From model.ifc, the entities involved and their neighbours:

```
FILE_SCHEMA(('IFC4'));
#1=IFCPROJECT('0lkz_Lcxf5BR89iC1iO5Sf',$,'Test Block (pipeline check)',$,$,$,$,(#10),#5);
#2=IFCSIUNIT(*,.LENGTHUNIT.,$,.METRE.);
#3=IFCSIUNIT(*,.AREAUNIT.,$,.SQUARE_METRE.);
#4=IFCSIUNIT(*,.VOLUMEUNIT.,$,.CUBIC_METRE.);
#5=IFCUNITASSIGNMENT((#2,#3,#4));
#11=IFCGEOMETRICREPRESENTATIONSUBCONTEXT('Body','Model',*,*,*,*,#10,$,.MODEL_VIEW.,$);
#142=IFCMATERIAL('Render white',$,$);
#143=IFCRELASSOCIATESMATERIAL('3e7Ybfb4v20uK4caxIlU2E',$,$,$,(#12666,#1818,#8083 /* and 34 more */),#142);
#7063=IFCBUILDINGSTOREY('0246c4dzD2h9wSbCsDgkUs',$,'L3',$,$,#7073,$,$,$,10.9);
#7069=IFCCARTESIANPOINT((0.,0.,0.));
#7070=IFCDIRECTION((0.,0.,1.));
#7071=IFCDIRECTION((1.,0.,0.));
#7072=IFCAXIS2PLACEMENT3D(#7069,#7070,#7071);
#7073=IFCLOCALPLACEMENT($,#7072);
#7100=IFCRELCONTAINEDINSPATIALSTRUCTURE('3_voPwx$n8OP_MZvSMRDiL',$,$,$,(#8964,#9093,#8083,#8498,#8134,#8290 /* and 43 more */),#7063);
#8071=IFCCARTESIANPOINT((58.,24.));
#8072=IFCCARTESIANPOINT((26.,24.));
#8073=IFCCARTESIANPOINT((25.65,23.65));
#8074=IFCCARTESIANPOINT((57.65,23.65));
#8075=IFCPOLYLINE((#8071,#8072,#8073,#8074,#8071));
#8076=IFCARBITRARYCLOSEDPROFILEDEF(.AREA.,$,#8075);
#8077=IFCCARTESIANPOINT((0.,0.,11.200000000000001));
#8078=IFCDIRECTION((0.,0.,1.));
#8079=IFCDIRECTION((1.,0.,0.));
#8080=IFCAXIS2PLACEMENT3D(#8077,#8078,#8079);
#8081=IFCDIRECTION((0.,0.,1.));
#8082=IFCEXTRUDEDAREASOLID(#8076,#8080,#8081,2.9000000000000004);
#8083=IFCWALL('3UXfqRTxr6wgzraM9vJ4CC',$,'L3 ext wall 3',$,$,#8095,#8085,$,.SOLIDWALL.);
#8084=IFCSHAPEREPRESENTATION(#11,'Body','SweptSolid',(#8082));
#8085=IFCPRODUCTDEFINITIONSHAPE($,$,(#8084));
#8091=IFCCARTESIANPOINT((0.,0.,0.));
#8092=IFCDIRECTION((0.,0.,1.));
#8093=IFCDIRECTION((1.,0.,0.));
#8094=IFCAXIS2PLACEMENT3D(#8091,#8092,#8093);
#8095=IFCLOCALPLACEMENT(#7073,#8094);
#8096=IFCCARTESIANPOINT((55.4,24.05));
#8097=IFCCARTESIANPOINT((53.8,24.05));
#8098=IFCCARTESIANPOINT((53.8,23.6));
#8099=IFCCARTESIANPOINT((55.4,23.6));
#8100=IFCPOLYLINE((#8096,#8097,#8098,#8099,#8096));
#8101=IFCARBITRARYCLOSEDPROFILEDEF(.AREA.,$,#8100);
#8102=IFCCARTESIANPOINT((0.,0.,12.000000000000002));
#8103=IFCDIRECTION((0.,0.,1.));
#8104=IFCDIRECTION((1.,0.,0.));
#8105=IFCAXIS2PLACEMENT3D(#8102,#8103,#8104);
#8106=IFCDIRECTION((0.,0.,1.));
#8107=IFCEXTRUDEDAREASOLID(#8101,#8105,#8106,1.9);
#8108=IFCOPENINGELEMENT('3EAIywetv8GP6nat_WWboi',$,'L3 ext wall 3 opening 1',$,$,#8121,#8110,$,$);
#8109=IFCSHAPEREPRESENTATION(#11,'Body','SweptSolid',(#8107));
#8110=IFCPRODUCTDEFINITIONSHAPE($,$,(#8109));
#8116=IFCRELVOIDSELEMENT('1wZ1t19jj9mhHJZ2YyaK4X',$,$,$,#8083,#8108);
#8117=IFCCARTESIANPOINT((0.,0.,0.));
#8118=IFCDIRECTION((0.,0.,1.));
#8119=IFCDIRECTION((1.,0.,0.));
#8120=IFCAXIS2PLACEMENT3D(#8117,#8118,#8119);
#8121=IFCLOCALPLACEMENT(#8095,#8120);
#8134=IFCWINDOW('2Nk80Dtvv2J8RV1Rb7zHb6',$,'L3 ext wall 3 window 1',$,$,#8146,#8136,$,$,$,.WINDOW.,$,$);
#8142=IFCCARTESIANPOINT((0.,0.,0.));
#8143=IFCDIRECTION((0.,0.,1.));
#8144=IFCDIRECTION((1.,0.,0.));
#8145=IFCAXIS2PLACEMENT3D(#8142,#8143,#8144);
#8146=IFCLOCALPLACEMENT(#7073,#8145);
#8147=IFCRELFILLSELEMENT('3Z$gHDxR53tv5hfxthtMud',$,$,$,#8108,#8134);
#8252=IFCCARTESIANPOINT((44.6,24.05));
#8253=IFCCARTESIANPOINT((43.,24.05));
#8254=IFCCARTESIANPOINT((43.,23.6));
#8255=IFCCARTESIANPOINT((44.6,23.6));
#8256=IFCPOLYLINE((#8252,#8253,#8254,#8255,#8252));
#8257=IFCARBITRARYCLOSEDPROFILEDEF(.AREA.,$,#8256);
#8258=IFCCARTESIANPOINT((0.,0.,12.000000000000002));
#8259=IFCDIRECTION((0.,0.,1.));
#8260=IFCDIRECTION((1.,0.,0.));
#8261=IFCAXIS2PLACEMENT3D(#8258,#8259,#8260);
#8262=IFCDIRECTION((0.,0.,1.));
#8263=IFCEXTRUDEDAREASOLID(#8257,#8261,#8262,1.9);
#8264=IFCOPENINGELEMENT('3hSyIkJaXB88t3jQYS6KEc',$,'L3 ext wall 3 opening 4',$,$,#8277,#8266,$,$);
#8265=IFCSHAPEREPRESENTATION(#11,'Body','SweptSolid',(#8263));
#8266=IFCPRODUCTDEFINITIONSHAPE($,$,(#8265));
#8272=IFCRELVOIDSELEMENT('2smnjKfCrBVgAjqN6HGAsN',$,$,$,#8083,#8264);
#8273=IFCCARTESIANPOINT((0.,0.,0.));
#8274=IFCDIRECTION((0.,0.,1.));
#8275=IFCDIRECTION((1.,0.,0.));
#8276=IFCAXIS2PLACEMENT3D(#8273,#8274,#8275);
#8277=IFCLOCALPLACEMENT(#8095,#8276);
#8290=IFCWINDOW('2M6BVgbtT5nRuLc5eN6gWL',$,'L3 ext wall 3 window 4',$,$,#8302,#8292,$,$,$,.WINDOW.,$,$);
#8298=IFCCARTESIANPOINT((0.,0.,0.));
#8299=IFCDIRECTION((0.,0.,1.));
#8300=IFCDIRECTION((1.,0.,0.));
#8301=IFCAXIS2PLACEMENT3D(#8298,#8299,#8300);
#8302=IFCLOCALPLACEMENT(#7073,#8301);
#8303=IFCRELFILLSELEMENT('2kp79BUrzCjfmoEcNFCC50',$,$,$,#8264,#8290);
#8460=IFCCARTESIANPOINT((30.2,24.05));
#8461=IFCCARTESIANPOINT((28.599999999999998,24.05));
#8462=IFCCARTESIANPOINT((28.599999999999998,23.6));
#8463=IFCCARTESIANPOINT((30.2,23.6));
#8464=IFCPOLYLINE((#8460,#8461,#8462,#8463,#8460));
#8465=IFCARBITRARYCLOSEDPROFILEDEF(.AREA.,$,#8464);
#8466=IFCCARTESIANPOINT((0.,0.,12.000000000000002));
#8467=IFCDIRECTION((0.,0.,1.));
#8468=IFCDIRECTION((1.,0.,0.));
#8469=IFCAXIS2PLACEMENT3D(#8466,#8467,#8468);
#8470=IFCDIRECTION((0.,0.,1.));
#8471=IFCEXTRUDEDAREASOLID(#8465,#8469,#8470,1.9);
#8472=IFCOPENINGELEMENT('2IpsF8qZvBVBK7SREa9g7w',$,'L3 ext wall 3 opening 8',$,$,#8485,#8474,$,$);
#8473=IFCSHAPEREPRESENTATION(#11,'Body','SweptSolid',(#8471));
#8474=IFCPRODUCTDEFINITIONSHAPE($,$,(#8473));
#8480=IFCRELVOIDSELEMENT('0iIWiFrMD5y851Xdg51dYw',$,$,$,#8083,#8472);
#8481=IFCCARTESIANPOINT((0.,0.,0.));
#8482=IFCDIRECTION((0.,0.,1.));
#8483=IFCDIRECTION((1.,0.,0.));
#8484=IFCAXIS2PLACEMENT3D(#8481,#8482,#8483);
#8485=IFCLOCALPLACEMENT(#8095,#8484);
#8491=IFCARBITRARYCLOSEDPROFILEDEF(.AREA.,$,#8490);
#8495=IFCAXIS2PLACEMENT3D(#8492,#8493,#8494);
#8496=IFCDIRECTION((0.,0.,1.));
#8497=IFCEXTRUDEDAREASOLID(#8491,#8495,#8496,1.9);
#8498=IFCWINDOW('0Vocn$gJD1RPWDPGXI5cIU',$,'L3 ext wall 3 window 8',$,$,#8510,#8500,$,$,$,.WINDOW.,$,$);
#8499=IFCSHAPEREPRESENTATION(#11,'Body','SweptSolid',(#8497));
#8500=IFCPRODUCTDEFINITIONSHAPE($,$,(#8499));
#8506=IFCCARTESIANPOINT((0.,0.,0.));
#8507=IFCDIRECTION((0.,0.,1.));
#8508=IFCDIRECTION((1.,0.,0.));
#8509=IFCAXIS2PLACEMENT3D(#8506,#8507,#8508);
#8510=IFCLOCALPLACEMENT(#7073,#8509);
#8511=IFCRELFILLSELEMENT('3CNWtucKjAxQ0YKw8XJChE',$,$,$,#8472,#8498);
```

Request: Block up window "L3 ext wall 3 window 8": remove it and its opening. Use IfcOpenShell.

```python
import ifcopenshell
import ifcopenshell.api.feature
import ifcopenshell.api.root
import ifcopenshell.geom
import ifcopenshell.util.shape

model = ifcopenshell.open("model.ifc")
settings = ifcopenshell.geom.settings()


def volume(element):
    """Net volume in cubic metres, openings subtracted."""
    shape = ifcopenshell.geom.create_shape(settings, element)
    return ifcopenshell.util.shape.get_volume(shape.geometry)


window = model.by_guid("0Vocn$gJD1RPWDPGXI5cIU")
opening = window.FillsVoids[0].RelatingOpeningElement
wall = opening.VoidsElements[0].RelatingBuildingElement
before = volume(wall)

ifcopenshell.api.root.remove_product(model, product=window)
ifcopenshell.api.feature.remove_feature(model, feature=opening)

after = volume(wall)

print(f"wall volume {before:.3f} -> {after:.3f} m3")

model.write("model_v2.ifc")
```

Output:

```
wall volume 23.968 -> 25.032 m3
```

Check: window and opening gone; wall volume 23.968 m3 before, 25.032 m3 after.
